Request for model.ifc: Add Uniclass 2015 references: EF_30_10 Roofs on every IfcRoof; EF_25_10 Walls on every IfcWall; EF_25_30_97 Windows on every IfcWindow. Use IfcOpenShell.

First a look at what the model holds.

```python
import ifcopenshell

model = ifcopenshell.open("model.ifc")
print(model.schema)
print("classifications:", [c.Name for c in model.by_type("IfcClassification")])
for ifc_class in ("IfcDoor", "IfcRoof", "IfcStair", "IfcWall", "IfcWindow"):
    print(ifc_class, len(model.by_type(ifc_class)))
```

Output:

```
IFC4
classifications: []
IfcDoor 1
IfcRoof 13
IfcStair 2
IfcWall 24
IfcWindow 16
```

```python
import ifcopenshell
import ifcopenshell.api.classification

model = ifcopenshell.open("model.ifc")

system = ifcopenshell.api.classification.add_classification(model, classification="Uniclass 2015")

codes = {
    "IfcRoof": ("EF_30_10", "Roofs"),
    "IfcWall": ("EF_25_10", "Walls"),
    "IfcWindow": ("EF_25_30_97", "Windows"),
}
for ifc_class, (code, name) in codes.items():
    products = model.by_type(ifc_class)
    ifcopenshell.api.classification.add_reference(
        model, products=products, classification=system, identification=code, name=name
    )
    print(code, len(products))

model.write("model-out.ifc")
```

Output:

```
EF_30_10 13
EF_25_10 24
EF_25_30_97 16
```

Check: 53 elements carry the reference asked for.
